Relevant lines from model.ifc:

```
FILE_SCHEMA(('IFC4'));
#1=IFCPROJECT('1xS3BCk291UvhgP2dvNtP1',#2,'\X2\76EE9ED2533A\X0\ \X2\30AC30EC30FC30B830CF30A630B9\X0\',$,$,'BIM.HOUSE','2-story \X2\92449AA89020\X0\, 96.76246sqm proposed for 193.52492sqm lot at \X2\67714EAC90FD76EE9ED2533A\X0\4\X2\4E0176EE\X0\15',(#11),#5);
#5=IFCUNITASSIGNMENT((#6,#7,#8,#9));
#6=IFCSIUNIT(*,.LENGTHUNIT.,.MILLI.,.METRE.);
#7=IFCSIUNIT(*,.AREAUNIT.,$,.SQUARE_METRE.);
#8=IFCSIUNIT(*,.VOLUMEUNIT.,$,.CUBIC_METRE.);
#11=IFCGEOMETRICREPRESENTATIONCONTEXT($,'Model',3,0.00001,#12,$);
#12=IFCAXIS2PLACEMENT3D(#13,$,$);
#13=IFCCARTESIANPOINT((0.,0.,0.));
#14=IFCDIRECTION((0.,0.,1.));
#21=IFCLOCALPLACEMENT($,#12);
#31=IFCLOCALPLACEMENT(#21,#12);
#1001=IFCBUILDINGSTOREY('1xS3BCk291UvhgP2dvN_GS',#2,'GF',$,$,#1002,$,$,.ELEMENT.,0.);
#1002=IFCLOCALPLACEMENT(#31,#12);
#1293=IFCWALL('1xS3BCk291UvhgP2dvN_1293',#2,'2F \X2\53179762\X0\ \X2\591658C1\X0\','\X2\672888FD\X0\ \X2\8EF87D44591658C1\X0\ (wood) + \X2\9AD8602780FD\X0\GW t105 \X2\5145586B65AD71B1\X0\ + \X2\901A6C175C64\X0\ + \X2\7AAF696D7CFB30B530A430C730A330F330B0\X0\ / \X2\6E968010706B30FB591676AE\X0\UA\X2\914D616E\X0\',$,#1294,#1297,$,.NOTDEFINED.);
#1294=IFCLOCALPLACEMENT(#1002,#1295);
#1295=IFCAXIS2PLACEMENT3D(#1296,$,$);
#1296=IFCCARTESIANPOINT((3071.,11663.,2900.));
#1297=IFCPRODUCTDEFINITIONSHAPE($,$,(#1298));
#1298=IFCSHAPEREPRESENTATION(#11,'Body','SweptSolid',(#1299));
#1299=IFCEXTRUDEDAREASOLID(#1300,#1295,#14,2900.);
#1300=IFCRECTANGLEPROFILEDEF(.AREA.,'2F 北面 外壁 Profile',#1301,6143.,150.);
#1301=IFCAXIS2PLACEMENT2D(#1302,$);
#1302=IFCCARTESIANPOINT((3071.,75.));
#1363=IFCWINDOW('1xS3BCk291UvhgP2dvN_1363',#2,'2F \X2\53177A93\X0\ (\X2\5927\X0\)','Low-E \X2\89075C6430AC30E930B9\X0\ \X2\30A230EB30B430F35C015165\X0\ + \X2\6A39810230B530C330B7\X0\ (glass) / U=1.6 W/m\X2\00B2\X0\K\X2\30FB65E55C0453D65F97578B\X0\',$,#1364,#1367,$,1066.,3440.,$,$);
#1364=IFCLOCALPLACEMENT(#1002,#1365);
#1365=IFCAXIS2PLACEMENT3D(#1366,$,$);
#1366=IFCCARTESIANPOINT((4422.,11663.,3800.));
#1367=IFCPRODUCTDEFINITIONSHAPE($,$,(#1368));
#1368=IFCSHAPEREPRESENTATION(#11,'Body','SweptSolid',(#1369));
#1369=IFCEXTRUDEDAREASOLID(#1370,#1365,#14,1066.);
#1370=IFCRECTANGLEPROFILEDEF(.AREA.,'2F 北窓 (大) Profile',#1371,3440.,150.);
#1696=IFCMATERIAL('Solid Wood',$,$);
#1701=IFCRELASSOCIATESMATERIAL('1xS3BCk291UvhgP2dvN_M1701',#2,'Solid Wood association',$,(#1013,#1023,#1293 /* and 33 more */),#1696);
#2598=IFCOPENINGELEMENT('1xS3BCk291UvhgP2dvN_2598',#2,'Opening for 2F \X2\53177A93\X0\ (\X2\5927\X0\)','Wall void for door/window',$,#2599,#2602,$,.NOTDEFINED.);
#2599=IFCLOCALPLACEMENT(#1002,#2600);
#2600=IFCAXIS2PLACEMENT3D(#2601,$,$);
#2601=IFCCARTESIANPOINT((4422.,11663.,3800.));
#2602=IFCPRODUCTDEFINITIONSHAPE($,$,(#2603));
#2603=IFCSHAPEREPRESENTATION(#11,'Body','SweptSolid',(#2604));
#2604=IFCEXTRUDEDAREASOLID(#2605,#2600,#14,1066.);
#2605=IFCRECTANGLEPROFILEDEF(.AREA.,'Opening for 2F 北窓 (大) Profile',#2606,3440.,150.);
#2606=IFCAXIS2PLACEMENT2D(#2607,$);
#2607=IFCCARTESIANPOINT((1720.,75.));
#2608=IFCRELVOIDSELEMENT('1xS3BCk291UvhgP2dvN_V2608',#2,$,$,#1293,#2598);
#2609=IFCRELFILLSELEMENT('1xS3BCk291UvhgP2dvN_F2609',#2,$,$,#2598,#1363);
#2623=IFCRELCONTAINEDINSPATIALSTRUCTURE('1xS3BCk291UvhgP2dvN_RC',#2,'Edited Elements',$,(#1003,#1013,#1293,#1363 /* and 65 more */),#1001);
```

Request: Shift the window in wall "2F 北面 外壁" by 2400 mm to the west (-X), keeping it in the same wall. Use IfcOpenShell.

```python
import ifcopenshell
import ifcopenshell.api.geometry
import ifcopenshell.util.placement
import ifcopenshell.util.unit

model = ifcopenshell.open("model.ifc")
unit_scale = ifcopenshell.util.unit.calculate_unit_scale(model)

window = model.by_guid("1xS3BCk291UvhgP2dvN_1363")
opening = window.FillsVoids[0].RelatingOpeningElement
wall = opening.VoidsElements[0].RelatingBuildingElement

wall_matrix = ifcopenshell.util.placement.get_local_placement(wall.ObjectPlacement)
shift = wall_matrix[:3, 0] * -2.4 / unit_scale
before = ifcopenshell.util.placement.get_local_placement(window.ObjectPlacement)[:3, 3].copy()

# The window is not placed relative to its opening, so move both.
for product in (opening, window):
    matrix = ifcopenshell.util.placement.get_local_placement(product.ObjectPlacement)
    matrix[:3, 3] += shift
    ifcopenshell.api.geometry.edit_object_placement(model, product=product, matrix=matrix, is_si=False)

after = ifcopenshell.util.placement.get_local_placement(window.ObjectPlacement)[:3, 3]
print("window moved by", (after - before).round(3) + 0.0)

model.write("model_rev.ifc")
```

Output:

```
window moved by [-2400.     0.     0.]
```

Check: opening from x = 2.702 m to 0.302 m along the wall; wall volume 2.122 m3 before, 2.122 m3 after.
